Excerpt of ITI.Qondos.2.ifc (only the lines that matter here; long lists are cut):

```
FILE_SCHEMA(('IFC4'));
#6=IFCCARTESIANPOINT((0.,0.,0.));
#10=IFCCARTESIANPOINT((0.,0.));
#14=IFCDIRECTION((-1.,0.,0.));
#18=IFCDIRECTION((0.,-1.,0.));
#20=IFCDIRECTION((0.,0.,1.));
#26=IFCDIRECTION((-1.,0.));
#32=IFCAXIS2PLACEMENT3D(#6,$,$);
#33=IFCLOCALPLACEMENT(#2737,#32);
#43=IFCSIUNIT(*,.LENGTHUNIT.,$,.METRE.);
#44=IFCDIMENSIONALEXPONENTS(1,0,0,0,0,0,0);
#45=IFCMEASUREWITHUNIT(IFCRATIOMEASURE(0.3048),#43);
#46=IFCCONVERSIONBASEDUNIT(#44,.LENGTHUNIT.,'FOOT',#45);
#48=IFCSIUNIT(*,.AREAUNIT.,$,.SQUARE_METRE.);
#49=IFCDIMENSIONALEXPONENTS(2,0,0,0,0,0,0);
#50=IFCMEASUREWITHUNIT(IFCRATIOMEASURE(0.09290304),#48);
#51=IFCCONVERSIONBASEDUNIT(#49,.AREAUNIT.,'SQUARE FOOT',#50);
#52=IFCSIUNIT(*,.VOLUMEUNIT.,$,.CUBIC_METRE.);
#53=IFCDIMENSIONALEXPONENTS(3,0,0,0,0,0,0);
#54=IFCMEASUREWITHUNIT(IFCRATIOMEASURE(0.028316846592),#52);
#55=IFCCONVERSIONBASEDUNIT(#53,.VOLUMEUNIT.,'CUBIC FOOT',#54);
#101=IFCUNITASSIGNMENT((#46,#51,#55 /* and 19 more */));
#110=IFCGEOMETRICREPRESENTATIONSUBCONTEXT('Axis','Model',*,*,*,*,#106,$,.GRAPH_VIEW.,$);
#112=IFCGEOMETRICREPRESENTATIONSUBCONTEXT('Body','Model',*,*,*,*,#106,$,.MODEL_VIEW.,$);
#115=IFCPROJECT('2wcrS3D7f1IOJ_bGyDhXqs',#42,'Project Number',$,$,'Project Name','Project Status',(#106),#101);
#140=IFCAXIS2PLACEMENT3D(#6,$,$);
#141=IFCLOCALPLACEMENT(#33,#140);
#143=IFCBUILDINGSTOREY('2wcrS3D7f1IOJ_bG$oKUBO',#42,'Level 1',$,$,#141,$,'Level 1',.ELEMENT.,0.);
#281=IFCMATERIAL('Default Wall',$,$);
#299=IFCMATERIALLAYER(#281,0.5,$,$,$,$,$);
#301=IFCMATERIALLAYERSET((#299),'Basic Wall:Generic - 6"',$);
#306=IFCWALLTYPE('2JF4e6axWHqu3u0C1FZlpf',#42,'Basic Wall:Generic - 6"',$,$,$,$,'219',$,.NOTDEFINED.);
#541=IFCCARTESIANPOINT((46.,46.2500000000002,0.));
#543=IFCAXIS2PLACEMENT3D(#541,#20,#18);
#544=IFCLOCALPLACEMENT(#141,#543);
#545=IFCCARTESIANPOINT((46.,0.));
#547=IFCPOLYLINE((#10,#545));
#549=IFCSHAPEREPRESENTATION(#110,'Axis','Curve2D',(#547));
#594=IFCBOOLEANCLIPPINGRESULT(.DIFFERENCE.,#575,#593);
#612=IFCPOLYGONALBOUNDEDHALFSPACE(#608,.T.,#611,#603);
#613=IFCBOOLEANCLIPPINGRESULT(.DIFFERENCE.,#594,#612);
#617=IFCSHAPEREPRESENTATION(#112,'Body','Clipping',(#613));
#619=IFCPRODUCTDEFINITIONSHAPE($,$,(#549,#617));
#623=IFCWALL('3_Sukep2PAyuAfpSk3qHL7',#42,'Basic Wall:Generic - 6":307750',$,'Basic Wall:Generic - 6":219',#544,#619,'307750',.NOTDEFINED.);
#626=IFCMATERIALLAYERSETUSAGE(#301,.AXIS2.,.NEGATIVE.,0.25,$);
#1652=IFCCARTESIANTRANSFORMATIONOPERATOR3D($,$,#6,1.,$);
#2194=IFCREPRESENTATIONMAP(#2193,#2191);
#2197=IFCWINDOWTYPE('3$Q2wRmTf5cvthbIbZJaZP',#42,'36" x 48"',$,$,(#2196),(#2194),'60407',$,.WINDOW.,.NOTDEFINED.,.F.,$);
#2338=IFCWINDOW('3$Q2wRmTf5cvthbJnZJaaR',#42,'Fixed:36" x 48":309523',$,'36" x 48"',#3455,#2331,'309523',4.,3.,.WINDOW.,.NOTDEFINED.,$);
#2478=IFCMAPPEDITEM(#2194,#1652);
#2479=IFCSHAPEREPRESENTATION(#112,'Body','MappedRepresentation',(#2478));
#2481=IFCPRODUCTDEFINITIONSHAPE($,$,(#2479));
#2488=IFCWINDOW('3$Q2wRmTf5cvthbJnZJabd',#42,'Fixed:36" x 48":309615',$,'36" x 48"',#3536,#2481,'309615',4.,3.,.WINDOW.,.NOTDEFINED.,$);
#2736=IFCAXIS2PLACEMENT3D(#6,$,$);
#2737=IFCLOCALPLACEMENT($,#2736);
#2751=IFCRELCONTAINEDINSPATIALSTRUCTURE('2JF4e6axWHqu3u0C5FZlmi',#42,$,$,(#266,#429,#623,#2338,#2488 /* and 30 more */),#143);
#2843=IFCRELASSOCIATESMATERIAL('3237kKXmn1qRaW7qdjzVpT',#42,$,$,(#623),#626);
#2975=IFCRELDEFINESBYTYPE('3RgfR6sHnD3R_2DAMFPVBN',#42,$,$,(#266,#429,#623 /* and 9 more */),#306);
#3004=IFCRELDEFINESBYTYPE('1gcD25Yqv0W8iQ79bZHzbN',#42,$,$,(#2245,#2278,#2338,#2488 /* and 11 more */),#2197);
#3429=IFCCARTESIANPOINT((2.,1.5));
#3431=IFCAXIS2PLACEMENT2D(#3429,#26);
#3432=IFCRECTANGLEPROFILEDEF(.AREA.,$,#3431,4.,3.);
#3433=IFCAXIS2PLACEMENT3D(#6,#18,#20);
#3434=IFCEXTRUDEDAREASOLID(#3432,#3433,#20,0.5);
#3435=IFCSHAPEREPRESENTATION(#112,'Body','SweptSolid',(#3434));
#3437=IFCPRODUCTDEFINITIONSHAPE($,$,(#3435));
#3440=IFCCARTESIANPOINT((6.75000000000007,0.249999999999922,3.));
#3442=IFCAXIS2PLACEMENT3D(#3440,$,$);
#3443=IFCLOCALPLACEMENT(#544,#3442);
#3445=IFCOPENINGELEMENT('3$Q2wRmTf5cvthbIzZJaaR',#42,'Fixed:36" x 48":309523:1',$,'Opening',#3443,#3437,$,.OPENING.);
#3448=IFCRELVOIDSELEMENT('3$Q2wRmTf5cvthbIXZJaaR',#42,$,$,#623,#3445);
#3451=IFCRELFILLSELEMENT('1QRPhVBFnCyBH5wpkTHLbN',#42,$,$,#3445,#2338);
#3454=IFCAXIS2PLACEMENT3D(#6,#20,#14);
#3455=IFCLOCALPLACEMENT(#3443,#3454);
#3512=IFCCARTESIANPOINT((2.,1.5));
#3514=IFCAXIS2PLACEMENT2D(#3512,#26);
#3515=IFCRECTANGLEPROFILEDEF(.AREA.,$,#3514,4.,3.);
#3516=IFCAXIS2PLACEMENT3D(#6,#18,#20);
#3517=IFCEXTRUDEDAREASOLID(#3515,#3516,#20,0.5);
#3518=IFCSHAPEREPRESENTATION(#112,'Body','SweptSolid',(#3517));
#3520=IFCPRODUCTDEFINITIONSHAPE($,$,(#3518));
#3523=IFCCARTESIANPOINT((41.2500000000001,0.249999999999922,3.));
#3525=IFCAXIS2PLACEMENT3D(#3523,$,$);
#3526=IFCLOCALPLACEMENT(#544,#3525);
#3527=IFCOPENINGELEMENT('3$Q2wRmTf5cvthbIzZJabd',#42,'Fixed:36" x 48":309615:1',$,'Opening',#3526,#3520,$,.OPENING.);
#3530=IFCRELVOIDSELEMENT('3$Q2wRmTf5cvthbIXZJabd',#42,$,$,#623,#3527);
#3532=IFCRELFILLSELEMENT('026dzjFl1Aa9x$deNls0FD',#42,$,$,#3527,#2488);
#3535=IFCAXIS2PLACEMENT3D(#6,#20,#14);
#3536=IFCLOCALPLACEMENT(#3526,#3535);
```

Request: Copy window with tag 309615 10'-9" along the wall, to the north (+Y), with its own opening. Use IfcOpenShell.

```python
import ifcopenshell
import ifcopenshell.api.feature
import ifcopenshell.api.geometry
import ifcopenshell.api.root
import ifcopenshell.geom
import ifcopenshell.util.element
import ifcopenshell.util.placement
import ifcopenshell.util.shape
import ifcopenshell.util.unit

model = ifcopenshell.open("ITI.Qondos.2.ifc")
unit_scale = ifcopenshell.util.unit.calculate_unit_scale(model)
settings = ifcopenshell.geom.settings()


def volume(element):
    """Net volume in cubic metres, openings subtracted."""
    shape = ifcopenshell.geom.create_shape(settings, element)
    return ifcopenshell.util.shape.get_volume(shape.geometry)


def reuse_history(source, copy):
    """copy_class also copies each property set's owner history, people and application; keep the originals."""
    for rel in copy.IsDefinedBy:
        if rel.is_a("IfcRelDefinesByProperties") and (history := rel.RelatingPropertyDefinition.OwnerHistory):
            rel.RelatingPropertyDefinition.OwnerHistory = source.OwnerHistory
            ifcopenshell.util.element.remove_deep2(model, history)


window = model.by_guid("3$Q2wRmTf5cvthbJnZJabd")
opening = window.FillsVoids[0].RelatingOpeningElement
wall = opening.VoidsElements[0].RelatingBuildingElement
before = volume(wall)
shift = ifcopenshell.util.placement.get_local_placement(wall.ObjectPlacement)[:3, 0] * -129 * 0.0254 / unit_scale

# copy_class copies the void relationship, type, container and properties, but no geometry.
new_opening = ifcopenshell.api.root.copy_class(model, product=opening)
new_opening.Representation = ifcopenshell.util.element.copy_deep(
    model, opening.Representation, exclude=["IfcGeometricRepresentationContext", "IfcRepresentationMap"]
)
new_opening.Name = 'Fixed:36" x 48"'
new_window = ifcopenshell.api.root.copy_class(model, product=window)
new_window.Representation = ifcopenshell.util.element.copy_deep(
    model, window.Representation, exclude=["IfcGeometricRepresentationContext", "IfcRepresentationMap"]
)
new_window.Name = 'Fixed:36" x 48"'
new_window.Tag = None
reuse_history(window, new_window)
ifcopenshell.api.feature.add_filling(model, opening=new_opening, element=new_window)

for old, new in ((opening, new_opening), (window, new_window)):
    matrix = ifcopenshell.util.placement.get_local_placement(old.ObjectPlacement)
    matrix[:3, 3] += shift
    ifcopenshell.api.geometry.edit_object_placement(model, product=new, matrix=matrix, is_si=False)

after = volume(wall)

print(f"wall volume {before:.3f} -> {after:.3f} m3")

model.write("ITI.Qondos.2_v2.ifc")
```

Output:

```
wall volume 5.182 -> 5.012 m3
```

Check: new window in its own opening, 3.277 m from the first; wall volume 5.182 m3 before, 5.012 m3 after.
